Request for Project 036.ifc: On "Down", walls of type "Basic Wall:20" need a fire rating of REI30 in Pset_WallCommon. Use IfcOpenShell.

First a look at what the model holds.

```python
import ifcopenshell
import ifcopenshell.util.element

model = ifcopenshell.open("Project 036.ifc")
print(model.schema)
storey = next(s for s in model.by_type("IfcBuildingStorey") if s.Name == "Down")
walls = [e for e in ifcopenshell.util.element.get_decomposition(storey) if e.is_a("IfcWall")]
seen = {}
for e in walls:
    element_type = ifcopenshell.util.element.get_type(e)
    key = (element_type.Name if element_type != e and element_type else None, ifcopenshell.util.element.get_pset(e, "Pset_WallCommon", "FireRating"))
    seen[key] = seen.get(key, 0) + 1
for (name, value), count in sorted(seen.items(), key=str):
    print(count, "x", name, "|", value)
```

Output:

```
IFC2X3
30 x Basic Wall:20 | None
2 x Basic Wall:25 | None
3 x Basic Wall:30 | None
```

```python
import ifcopenshell
import ifcopenshell.api.pset
import ifcopenshell.util.element

model = ifcopenshell.open("Project 036.ifc")

storey = next(s for s in model.by_type("IfcBuildingStorey") if s.Name == "Down")
walls = [e for e in ifcopenshell.util.element.get_decomposition(storey) if e.is_a("IfcWall")]

count = 0
for e in walls:
    element_type = ifcopenshell.util.element.get_type(e)
    if element_type in (None, e) or element_type.Name != "Basic Wall:20":
        continue
    # add_pset returns the element's existing set when there is one.
    pset = ifcopenshell.api.pset.add_pset(model, product=e, name="Pset_WallCommon")
    ifcopenshell.api.pset.edit_pset(model, pset=pset, properties={"FireRating": "REI30"})
    count += 1

print(count, "walls updated")

model.write("Project 036_v2.ifc")
```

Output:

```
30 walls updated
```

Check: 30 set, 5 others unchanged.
